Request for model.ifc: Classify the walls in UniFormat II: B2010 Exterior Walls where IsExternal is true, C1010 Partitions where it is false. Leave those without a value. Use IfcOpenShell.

First a look at what the model holds.

```python
import ifcopenshell
import ifcopenshell.util.element

model = ifcopenshell.open("model.ifc")
print(model.schema)
print("classifications:", [c.Name for c in model.by_type("IfcClassification")])
values = [ifcopenshell.util.element.get_pset(e, "Pset_WallCommon", "IsExternal") for e in model.by_type("IfcWall")]
for value in (True, False, None):
    print("IsExternal", value, values.count(value))
```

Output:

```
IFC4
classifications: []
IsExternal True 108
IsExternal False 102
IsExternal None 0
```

```python
import ifcopenshell
import ifcopenshell.api.classification
import ifcopenshell.util.element

model = ifcopenshell.open("model.ifc")

system = ifcopenshell.api.classification.add_classification(model, classification="UniFormat II")

walls = model.by_type("IfcWall")
external = {e: ifcopenshell.util.element.get_pset(e, "Pset_WallCommon", "IsExternal") for e in walls}
for flag, code, name in ((True, "B2010", "Exterior Walls"), (False, "C1010", "Partitions")):
    products = [e for e in walls if external[e] is flag]
    ifcopenshell.api.classification.add_reference(
        model, products=products, classification=system, identification=code, name=name
    )
    print(code, len(products))

model.write("model_edited.ifc")
```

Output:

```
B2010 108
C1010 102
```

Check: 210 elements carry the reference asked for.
